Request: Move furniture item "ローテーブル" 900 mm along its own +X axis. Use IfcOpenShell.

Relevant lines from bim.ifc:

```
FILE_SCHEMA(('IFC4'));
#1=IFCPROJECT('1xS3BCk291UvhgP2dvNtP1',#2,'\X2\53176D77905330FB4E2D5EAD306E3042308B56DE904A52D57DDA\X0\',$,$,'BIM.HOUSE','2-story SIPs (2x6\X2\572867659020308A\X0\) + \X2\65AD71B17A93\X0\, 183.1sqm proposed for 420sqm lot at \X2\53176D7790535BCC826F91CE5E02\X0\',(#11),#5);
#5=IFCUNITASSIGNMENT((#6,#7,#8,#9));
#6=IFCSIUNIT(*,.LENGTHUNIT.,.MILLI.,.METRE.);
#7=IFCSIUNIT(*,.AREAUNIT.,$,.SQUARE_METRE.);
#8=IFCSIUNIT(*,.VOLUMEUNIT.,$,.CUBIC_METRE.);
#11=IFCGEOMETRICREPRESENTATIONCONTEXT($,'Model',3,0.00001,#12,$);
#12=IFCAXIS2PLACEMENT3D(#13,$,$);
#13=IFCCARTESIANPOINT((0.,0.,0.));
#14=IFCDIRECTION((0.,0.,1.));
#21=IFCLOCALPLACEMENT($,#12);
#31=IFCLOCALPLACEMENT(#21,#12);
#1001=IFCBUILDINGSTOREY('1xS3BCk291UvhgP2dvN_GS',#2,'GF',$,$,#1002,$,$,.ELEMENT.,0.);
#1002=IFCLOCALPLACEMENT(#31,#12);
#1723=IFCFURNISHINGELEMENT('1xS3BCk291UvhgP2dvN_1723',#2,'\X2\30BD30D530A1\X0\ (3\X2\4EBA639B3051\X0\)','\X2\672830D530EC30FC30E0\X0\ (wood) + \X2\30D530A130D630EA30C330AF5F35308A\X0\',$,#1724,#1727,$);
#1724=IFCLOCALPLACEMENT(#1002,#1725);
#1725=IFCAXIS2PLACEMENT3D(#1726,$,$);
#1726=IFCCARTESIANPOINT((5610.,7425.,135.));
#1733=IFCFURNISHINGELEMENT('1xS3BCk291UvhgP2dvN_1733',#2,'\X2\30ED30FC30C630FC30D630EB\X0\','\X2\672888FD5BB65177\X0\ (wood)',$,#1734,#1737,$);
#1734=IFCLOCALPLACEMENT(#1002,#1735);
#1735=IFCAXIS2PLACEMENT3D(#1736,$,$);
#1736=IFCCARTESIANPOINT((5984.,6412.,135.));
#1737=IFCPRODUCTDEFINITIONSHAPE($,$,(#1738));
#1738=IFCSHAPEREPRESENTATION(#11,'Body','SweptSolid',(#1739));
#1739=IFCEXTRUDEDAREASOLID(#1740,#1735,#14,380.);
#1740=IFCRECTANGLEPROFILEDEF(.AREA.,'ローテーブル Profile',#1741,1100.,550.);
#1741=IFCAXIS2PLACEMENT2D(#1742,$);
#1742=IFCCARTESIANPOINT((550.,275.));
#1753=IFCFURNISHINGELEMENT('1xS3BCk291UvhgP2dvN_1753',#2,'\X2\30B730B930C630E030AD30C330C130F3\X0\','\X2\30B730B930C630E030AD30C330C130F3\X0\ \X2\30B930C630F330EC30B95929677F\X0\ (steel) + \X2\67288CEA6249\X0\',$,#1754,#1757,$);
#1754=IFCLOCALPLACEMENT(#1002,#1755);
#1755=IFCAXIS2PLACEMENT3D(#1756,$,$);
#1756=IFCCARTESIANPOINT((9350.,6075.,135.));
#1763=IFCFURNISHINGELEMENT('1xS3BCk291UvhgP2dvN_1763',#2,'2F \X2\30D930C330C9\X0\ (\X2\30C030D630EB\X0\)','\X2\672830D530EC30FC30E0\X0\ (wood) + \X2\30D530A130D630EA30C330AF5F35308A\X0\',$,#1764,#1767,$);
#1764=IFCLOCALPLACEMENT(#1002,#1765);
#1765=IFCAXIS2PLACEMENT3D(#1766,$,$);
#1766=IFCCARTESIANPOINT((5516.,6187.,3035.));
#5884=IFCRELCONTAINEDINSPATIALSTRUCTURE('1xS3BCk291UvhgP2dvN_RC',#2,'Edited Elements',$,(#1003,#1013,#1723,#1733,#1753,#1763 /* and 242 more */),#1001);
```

```python
import ifcopenshell
import ifcopenshell.api.geometry
import ifcopenshell.util.placement
import ifcopenshell.util.unit

model = ifcopenshell.open("bim.ifc")
unit_scale = ifcopenshell.util.unit.calculate_unit_scale(model)

item = model.by_guid("1xS3BCk291UvhgP2dvN_1733")
matrix = ifcopenshell.util.placement.get_local_placement(item.ObjectPlacement)
matrix[:3, 3] += matrix[:3, 0] * 0.9 / unit_scale
ifcopenshell.api.geometry.edit_object_placement(model, product=item, matrix=matrix, is_si=False)

print(ifcopenshell.util.placement.get_local_placement(item.ObjectPlacement).round(3) + 0.0)

model.write("bim_edited.ifc")
```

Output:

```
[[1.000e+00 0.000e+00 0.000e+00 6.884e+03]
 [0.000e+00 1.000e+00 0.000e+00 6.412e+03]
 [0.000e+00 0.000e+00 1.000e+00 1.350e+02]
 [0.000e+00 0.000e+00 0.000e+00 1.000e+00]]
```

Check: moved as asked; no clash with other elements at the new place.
